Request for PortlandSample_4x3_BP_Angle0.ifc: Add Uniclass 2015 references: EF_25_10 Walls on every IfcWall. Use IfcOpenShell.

First a look at what the model holds.

```python
import ifcopenshell

model = ifcopenshell.open("PortlandSample_4x3_BP_Angle0.ifc")
print(model.schema)
print("classifications:", [c.Name for c in model.by_type("IfcClassification")])
for ifc_class in ("IfcDoor", "IfcRoof", "IfcStair", "IfcWall", "IfcWindow"):
    print(ifc_class, len(model.by_type(ifc_class)))
```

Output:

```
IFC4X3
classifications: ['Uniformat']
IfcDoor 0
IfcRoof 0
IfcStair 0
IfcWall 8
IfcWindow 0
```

```python
import ifcopenshell
import ifcopenshell.api.classification

model = ifcopenshell.open("PortlandSample_4x3_BP_Angle0.ifc")

system = ifcopenshell.api.classification.add_classification(model, classification="Uniclass 2015")

codes = {
    "IfcWall": ("EF_25_10", "Walls"),
}
for ifc_class, (code, name) in codes.items():
    products = model.by_type(ifc_class)
    ifcopenshell.api.classification.add_reference(
        model, products=products, classification=system, identification=code, name=name
    )
    print(code, len(products))

model.write("PortlandSample_4x3_BP_Angle0_updated.ifc")
```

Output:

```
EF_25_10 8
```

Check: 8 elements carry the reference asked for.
